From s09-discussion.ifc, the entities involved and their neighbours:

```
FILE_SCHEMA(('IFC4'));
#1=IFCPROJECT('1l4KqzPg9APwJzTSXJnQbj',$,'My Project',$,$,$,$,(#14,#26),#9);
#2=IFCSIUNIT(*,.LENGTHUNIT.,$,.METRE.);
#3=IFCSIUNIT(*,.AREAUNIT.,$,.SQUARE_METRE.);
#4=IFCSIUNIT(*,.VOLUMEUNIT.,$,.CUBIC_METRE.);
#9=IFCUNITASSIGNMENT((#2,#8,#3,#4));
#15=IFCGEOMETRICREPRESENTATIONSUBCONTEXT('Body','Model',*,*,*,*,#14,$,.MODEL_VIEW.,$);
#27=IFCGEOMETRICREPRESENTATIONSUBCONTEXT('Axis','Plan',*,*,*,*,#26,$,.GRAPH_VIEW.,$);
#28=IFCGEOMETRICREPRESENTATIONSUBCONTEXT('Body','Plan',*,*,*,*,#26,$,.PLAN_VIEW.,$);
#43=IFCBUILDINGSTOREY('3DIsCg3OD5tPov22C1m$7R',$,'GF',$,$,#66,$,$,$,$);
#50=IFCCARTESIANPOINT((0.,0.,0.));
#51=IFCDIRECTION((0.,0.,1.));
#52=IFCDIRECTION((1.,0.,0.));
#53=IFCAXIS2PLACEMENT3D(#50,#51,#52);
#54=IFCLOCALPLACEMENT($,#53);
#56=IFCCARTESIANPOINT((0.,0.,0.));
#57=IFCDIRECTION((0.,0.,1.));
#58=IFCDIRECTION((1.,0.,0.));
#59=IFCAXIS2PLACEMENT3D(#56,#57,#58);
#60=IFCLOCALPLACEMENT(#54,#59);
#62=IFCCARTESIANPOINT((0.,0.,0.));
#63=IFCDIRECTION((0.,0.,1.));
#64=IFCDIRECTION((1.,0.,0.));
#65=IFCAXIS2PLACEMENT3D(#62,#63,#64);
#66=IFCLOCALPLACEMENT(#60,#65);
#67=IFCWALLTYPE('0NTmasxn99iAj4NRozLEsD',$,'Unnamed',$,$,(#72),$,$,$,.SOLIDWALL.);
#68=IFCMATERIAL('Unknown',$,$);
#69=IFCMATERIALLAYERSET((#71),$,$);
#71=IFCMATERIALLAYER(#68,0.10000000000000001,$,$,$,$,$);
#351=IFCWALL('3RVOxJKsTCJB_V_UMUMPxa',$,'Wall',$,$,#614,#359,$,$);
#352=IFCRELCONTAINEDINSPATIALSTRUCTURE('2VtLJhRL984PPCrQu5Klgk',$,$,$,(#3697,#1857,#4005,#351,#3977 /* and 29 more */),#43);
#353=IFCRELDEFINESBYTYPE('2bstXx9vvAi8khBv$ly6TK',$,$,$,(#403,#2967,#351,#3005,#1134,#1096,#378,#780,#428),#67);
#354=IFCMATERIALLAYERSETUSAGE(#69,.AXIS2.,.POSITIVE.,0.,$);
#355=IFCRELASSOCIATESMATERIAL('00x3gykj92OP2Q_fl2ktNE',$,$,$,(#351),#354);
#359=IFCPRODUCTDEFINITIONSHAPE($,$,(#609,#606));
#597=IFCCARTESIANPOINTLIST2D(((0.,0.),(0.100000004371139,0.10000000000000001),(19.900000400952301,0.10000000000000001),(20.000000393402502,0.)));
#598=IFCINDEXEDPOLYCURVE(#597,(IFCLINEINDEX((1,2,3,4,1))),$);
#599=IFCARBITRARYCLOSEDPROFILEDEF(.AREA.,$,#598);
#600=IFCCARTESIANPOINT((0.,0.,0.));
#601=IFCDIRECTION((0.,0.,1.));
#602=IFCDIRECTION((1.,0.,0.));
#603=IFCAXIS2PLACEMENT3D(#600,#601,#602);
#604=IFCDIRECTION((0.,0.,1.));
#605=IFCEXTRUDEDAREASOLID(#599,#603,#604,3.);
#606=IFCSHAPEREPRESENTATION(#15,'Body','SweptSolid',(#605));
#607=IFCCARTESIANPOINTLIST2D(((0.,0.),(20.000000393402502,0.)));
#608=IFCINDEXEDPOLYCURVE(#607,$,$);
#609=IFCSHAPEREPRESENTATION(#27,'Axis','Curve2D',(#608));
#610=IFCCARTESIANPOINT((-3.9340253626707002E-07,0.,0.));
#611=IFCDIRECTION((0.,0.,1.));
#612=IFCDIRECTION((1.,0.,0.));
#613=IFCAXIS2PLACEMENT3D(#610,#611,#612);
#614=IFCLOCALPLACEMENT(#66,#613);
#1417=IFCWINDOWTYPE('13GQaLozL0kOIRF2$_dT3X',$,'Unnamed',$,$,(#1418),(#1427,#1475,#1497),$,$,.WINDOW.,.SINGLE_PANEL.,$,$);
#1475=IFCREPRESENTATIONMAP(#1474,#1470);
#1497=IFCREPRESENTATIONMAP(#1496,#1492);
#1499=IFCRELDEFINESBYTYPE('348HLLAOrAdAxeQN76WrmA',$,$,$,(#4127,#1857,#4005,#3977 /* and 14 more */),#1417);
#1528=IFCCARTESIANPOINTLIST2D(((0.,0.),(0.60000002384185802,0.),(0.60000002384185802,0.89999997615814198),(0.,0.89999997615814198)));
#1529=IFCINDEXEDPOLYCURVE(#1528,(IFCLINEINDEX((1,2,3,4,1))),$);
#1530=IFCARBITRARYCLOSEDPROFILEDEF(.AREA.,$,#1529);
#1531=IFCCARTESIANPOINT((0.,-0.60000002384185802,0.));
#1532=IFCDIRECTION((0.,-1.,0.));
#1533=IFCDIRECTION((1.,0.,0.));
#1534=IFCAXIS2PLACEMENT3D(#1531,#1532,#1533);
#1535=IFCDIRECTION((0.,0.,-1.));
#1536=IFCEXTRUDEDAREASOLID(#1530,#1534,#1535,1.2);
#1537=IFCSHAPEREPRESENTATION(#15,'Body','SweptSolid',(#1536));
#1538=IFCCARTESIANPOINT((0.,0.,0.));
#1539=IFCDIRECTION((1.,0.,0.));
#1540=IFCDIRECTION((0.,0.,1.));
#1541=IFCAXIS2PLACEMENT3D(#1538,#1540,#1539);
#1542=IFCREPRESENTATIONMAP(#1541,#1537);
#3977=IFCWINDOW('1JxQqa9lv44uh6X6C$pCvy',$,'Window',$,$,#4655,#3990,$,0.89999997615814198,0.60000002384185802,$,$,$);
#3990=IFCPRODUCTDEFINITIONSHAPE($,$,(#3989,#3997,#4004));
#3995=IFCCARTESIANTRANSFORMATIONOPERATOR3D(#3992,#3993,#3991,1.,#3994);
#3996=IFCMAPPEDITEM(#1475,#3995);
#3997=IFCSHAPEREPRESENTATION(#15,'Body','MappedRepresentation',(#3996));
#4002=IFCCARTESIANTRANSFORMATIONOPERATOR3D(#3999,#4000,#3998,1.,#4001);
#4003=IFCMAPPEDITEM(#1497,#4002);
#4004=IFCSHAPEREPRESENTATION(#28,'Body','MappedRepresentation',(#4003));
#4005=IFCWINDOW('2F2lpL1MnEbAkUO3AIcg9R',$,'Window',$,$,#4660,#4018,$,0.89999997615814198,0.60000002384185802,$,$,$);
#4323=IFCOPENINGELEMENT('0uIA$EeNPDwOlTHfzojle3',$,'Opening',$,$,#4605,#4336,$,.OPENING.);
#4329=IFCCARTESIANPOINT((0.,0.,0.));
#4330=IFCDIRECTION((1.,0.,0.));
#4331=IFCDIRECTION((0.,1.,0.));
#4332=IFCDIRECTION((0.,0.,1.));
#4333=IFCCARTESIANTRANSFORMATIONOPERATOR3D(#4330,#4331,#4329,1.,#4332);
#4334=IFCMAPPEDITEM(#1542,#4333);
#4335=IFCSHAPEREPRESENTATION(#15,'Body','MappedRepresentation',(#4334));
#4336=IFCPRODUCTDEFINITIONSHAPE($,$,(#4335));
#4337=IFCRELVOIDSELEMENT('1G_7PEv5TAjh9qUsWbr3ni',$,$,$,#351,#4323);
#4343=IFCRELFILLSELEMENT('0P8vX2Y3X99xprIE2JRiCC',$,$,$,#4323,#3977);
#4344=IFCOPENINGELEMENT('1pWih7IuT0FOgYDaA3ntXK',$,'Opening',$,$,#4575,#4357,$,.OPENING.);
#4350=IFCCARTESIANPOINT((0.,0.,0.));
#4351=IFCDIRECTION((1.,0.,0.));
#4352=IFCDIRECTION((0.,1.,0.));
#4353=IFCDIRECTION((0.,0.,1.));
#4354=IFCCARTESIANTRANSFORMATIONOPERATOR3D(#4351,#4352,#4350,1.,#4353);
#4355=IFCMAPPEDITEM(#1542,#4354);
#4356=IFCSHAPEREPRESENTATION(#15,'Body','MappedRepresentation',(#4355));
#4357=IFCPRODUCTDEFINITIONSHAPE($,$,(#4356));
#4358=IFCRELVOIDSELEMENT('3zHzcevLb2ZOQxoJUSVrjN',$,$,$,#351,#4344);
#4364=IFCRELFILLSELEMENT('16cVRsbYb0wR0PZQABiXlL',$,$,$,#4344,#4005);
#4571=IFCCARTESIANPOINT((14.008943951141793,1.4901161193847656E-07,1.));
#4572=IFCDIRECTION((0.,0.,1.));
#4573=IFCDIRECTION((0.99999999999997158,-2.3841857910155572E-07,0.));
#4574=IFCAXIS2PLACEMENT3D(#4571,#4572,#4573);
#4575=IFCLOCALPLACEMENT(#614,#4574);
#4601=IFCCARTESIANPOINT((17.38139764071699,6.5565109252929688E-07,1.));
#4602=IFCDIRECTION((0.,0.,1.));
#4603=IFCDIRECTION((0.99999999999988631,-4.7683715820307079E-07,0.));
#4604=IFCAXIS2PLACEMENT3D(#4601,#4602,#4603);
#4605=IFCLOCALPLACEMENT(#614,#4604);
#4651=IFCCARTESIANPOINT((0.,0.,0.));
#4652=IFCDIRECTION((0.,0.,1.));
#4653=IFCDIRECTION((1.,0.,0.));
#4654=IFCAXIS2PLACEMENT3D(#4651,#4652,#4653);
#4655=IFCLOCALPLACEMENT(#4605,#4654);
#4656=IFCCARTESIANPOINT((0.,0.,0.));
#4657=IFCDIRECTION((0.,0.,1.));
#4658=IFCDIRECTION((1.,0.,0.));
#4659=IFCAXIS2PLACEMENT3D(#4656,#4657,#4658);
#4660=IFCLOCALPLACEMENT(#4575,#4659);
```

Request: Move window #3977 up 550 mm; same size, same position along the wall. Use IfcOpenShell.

```python
import numpy as np
import ifcopenshell
import ifcopenshell.api.geometry
import ifcopenshell.util.placement
import ifcopenshell.util.unit

model = ifcopenshell.open("s09-discussion.ifc")
unit_scale = ifcopenshell.util.unit.calculate_unit_scale(model)

window = model.by_id(3977)
opening = window.FillsVoids[0].RelatingOpeningElement
dz = 0.55

shift = np.array([0.0, 0.0, dz])
# The window is placed relative to its opening, so it follows when the opening moves.
matrix = ifcopenshell.util.placement.get_local_placement(opening.ObjectPlacement)
matrix[:3, 3] += shift
ifcopenshell.api.geometry.edit_object_placement(
    model, product=opening, matrix=matrix, is_si=False, should_transform_children=True
)

print(f"moved by {dz * unit_scale:+.3f} m")

model.write("s09-discussion-out.ifc")
```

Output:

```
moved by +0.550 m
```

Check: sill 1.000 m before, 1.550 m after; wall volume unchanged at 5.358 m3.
